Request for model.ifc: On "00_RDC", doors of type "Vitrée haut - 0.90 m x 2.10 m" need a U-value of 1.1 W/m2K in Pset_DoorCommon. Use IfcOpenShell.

First a look at what the model holds.

```python
import ifcopenshell
import ifcopenshell.util.element

model = ifcopenshell.open("model.ifc")
print(model.schema)
storey = next(s for s in model.by_type("IfcBuildingStorey") if s.Name == "00_RDC")
doors = [e for e in ifcopenshell.util.element.get_decomposition(storey) if e.is_a("IfcDoor")]
seen = {}
for e in doors:
    element_type = ifcopenshell.util.element.get_type(e)
    key = (element_type.Name if element_type != e and element_type else None, ifcopenshell.util.element.get_pset(e, "Pset_DoorCommon", "ThermalTransmittance"))
    seen[key] = seen.get(key, 0) + 1
for (name, value), count in sorted(seen.items(), key=str):
    print(count, "x", name, "|", value)
```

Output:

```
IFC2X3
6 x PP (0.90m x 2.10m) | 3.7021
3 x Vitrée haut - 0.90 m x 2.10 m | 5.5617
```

```python
import ifcopenshell
import ifcopenshell.api.pset
import ifcopenshell.util.element

model = ifcopenshell.open("model.ifc")

storey = next(s for s in model.by_type("IfcBuildingStorey") if s.Name == "00_RDC")
doors = [e for e in ifcopenshell.util.element.get_decomposition(storey) if e.is_a("IfcDoor")]

count = 0
for e in doors:
    element_type = ifcopenshell.util.element.get_type(e)
    if element_type in (None, e) or element_type.Name != "Vitrée haut - 0.90 m x 2.10 m":
        continue
    # add_pset returns the element's existing set when there is one.
    pset = ifcopenshell.api.pset.add_pset(model, product=e, name="Pset_DoorCommon")
    ifcopenshell.api.pset.edit_pset(model, pset=pset, properties={"ThermalTransmittance": 1.1})
    count += 1

print(count, "doors updated")

model.write("model-out.ifc")
```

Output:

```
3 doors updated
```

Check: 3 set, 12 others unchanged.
